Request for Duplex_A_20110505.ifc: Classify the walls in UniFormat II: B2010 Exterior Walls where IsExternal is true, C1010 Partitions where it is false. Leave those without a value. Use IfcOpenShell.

First a look at what the model holds.

```python
import ifcopenshell
import ifcopenshell.util.element

model = ifcopenshell.open("Duplex_A_20110505.ifc")
print(model.schema)
print("classifications:", [c.Name for c in model.by_type("IfcClassification")])
values = [ifcopenshell.util.element.get_pset(e, "Pset_WallCommon", "IsExternal") for e in model.by_type("IfcWall")]
for value in (True, False, None):
    print("IsExternal", value, values.count(value))
```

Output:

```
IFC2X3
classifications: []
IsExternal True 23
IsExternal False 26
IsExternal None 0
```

```python
import ifcopenshell
import ifcopenshell.api.classification
import ifcopenshell.util.element

model = ifcopenshell.open("Duplex_A_20110505.ifc")

# IFC2X3 requires Source and Edition and has no link from the project to the system.
system = model.create_entity("IfcClassification", Source="ASTM", Edition="E1557", Name="UniFormat II")

walls = model.by_type("IfcWall")
external = {e: ifcopenshell.util.element.get_pset(e, "Pset_WallCommon", "IsExternal") for e in walls}
for flag, code, name in ((True, "B2010", "Exterior Walls"), (False, "C1010", "Partitions")):
    products = [e for e in walls if external[e] is flag]
    ifcopenshell.api.classification.add_reference(
        model, products=products, classification=system, identification=code, name=name
    )
    print(code, len(products))

model.write("Duplex_A_20110505_edited.ifc")
```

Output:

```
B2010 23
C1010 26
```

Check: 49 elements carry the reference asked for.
